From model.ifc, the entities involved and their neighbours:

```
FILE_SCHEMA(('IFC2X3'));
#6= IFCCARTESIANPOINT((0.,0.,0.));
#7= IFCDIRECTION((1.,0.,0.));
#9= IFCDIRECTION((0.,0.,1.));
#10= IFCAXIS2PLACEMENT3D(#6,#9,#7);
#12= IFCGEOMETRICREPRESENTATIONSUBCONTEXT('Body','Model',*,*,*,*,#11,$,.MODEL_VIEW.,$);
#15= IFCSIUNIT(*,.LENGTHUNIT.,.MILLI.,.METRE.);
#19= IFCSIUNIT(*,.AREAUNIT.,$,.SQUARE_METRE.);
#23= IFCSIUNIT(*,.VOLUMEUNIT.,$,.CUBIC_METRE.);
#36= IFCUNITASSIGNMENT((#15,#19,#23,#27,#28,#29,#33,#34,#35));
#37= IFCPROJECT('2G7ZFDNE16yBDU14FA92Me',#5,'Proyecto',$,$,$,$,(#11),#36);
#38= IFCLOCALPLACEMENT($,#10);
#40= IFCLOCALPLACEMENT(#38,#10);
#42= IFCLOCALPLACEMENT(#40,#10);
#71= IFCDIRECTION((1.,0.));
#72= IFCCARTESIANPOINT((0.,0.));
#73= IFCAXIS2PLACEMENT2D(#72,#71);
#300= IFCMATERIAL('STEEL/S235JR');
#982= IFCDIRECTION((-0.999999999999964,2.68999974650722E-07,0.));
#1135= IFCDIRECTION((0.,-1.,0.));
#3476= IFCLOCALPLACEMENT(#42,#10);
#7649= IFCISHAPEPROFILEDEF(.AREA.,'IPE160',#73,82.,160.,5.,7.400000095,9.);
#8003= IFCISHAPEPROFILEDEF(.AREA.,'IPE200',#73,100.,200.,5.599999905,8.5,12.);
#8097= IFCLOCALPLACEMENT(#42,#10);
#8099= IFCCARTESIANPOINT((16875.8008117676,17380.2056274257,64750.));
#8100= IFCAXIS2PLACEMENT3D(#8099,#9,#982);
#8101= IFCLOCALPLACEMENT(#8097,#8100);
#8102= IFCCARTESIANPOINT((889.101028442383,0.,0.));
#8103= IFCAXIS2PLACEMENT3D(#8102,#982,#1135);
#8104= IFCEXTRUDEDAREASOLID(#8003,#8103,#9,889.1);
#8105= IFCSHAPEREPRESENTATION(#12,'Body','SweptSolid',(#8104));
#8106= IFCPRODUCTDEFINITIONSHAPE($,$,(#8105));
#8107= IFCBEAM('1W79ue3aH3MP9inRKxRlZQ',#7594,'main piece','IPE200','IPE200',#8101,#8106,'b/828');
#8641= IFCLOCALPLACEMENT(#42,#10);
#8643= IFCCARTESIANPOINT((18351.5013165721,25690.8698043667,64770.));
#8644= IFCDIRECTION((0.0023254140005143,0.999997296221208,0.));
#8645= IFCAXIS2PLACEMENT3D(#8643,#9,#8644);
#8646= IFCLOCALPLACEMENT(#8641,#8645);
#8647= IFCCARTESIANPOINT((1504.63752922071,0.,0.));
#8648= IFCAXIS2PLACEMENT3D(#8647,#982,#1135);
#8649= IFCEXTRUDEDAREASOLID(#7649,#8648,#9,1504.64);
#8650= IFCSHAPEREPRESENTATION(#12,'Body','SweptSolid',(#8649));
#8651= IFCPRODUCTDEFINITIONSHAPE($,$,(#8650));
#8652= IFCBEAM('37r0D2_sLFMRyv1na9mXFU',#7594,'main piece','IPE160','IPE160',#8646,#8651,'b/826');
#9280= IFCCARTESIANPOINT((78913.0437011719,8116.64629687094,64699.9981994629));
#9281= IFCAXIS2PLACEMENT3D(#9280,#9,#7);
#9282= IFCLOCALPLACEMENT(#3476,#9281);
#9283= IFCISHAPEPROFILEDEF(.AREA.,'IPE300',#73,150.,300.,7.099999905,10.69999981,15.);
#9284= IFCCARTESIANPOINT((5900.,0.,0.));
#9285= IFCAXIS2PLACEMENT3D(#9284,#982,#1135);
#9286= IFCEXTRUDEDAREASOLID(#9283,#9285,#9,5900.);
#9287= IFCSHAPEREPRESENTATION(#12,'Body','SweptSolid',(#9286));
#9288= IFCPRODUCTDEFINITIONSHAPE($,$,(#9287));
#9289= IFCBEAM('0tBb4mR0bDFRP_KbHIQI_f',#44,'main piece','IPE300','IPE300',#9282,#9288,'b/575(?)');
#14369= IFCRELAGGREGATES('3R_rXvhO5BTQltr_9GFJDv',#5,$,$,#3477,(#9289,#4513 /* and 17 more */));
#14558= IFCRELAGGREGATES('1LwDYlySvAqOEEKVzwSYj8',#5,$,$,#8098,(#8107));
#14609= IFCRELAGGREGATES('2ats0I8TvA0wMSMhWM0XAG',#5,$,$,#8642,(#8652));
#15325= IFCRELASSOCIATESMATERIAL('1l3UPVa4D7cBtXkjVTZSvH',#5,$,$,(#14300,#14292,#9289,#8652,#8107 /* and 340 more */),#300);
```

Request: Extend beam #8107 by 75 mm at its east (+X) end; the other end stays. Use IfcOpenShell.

```python
import ifcopenshell
import ifcopenshell.util.representation

model = ifcopenshell.open("model.ifc")

member = model.by_guid("1W79ue3aH3MP9inRKxRlZQ")
change = 75.0

# The extrusion runs towards the end named, so only its depth changes.
body = ifcopenshell.util.representation.get_representation(member, "Model", "Body")
solid = body.Items[0]
old_length = solid.Depth
solid.Depth += change

print(f"length {old_length:g} -> {solid.Depth:g}")

model.write("model-out.ifc")
```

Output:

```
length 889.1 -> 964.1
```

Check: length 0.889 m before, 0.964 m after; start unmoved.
